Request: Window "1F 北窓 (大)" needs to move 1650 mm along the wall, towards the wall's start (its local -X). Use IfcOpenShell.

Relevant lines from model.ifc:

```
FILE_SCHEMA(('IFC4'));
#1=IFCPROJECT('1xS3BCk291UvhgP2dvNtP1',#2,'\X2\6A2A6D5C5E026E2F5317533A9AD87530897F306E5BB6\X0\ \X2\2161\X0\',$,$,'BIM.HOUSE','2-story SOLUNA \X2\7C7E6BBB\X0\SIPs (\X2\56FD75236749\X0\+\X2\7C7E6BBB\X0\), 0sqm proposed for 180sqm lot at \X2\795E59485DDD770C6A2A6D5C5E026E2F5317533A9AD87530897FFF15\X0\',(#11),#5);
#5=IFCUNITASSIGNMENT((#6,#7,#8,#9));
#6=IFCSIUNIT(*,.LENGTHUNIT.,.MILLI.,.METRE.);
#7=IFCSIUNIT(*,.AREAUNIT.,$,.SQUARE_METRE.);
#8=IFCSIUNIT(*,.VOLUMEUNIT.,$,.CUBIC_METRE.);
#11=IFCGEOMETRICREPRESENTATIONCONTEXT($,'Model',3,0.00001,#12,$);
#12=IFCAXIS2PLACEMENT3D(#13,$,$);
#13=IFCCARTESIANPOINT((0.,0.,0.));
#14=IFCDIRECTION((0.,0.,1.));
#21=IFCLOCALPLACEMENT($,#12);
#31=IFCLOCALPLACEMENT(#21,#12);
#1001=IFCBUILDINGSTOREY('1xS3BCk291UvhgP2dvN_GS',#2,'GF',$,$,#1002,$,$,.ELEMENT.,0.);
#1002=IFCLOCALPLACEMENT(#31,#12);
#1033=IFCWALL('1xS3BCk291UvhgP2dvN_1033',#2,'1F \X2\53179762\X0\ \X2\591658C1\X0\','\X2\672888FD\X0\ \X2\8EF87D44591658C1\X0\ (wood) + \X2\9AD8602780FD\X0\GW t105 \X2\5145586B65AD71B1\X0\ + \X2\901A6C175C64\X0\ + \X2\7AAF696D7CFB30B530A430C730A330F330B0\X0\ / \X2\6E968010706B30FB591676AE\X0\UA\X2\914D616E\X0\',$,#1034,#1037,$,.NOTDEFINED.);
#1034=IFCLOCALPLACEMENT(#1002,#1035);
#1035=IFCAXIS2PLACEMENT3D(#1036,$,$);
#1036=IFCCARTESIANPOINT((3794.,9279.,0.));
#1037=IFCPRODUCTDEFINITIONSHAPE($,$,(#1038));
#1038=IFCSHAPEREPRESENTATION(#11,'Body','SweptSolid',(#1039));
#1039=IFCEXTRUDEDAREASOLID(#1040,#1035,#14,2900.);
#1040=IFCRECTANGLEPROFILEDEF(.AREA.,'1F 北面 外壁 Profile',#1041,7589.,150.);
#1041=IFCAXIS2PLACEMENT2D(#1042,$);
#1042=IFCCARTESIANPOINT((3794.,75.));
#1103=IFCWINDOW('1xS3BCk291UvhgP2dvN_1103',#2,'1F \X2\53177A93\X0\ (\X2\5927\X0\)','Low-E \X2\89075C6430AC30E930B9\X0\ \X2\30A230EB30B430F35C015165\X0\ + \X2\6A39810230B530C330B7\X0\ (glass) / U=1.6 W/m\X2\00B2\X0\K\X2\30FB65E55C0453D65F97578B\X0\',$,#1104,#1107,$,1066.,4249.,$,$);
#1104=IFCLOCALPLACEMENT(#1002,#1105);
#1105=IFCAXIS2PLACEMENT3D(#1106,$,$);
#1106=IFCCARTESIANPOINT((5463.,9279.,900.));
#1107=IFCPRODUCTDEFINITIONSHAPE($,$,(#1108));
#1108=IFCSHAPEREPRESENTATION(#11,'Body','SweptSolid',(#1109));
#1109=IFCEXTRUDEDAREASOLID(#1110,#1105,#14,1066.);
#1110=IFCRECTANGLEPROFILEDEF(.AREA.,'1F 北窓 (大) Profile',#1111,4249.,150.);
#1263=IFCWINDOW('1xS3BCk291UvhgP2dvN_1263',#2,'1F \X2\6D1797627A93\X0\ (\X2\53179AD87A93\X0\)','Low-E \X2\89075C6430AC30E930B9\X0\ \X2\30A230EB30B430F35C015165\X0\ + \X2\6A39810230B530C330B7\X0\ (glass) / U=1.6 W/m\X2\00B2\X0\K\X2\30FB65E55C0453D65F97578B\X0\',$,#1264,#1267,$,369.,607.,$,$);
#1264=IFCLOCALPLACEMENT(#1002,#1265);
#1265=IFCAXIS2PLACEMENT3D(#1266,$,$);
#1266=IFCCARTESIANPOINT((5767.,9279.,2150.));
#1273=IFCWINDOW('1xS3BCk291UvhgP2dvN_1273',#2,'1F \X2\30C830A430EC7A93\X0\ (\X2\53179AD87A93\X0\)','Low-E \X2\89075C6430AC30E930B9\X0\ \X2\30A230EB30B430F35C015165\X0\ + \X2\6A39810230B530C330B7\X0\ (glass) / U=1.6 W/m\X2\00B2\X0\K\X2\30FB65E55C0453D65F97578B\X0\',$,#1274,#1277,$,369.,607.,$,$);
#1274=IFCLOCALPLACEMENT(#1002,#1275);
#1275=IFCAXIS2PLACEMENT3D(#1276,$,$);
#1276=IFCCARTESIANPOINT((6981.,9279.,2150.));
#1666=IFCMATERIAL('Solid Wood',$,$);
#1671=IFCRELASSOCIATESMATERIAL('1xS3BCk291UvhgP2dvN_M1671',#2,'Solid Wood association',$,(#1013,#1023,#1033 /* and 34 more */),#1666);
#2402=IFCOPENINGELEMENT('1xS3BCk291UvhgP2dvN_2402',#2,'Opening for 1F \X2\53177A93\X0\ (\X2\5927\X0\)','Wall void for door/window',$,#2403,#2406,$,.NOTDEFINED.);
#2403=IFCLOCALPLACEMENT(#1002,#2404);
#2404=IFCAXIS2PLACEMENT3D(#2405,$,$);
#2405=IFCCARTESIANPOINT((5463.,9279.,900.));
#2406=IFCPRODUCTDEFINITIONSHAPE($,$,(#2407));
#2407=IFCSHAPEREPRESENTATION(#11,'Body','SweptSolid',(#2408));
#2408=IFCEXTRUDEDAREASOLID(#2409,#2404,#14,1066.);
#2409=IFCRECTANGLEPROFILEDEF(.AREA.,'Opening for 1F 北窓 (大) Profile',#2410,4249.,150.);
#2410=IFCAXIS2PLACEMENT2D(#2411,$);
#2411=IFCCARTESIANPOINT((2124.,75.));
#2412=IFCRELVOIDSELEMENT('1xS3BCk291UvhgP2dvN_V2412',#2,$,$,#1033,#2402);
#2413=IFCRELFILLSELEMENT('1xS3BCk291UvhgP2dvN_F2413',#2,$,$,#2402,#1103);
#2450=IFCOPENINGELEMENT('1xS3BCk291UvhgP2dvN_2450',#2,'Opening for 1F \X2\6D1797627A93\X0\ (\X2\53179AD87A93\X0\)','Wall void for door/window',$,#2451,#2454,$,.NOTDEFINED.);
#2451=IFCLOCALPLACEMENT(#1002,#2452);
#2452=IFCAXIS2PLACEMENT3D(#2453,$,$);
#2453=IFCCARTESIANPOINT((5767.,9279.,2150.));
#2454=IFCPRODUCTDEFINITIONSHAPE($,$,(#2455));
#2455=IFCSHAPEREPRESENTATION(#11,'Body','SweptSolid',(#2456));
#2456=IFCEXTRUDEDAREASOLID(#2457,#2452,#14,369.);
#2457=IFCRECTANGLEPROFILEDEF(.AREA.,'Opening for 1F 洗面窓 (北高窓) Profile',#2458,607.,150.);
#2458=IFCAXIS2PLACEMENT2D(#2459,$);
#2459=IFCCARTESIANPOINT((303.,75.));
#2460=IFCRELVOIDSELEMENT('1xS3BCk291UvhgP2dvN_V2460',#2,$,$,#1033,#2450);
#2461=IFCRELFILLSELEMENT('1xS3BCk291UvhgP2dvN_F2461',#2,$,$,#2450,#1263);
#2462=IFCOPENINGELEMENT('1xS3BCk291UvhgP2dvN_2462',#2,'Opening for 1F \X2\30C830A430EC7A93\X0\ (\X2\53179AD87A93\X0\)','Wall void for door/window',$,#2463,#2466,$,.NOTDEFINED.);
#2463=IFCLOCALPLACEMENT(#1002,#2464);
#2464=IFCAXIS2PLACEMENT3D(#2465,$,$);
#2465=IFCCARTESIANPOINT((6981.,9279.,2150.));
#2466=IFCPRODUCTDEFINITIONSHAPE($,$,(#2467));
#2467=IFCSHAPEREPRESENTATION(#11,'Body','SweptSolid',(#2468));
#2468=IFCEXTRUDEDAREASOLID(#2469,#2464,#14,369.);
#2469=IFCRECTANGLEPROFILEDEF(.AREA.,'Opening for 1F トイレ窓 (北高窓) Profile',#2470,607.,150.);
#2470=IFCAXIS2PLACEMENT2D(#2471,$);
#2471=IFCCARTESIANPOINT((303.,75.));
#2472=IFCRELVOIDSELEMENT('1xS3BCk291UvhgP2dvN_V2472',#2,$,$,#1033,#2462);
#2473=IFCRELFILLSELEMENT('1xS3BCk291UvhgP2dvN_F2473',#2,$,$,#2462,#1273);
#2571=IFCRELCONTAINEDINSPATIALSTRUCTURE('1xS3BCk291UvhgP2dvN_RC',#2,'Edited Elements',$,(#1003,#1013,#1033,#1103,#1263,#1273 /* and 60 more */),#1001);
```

```python
import ifcopenshell
import ifcopenshell.api.geometry
import ifcopenshell.util.placement
import ifcopenshell.util.unit

model = ifcopenshell.open("model.ifc")
unit_scale = ifcopenshell.util.unit.calculate_unit_scale(model)

window = model.by_guid("1xS3BCk291UvhgP2dvN_1103")
opening = window.FillsVoids[0].RelatingOpeningElement
wall = opening.VoidsElements[0].RelatingBuildingElement

wall_matrix = ifcopenshell.util.placement.get_local_placement(wall.ObjectPlacement)
shift = wall_matrix[:3, 0] * -1.65 / unit_scale
before = ifcopenshell.util.placement.get_local_placement(window.ObjectPlacement)[:3, 3].copy()

# The window is not placed relative to its opening, so move both.
for product in (opening, window):
    matrix = ifcopenshell.util.placement.get_local_placement(product.ObjectPlacement)
    matrix[:3, 3] += shift
    ifcopenshell.api.geometry.edit_object_placement(model, product=product, matrix=matrix, is_si=False)

after = ifcopenshell.util.placement.get_local_placement(window.ObjectPlacement)[:3, 3]
print("window moved by", (after - before).round(3) + 0.0)

model.write("model_v2.ifc")
```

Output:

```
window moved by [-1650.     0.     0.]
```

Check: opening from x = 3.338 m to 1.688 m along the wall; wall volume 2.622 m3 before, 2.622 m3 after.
